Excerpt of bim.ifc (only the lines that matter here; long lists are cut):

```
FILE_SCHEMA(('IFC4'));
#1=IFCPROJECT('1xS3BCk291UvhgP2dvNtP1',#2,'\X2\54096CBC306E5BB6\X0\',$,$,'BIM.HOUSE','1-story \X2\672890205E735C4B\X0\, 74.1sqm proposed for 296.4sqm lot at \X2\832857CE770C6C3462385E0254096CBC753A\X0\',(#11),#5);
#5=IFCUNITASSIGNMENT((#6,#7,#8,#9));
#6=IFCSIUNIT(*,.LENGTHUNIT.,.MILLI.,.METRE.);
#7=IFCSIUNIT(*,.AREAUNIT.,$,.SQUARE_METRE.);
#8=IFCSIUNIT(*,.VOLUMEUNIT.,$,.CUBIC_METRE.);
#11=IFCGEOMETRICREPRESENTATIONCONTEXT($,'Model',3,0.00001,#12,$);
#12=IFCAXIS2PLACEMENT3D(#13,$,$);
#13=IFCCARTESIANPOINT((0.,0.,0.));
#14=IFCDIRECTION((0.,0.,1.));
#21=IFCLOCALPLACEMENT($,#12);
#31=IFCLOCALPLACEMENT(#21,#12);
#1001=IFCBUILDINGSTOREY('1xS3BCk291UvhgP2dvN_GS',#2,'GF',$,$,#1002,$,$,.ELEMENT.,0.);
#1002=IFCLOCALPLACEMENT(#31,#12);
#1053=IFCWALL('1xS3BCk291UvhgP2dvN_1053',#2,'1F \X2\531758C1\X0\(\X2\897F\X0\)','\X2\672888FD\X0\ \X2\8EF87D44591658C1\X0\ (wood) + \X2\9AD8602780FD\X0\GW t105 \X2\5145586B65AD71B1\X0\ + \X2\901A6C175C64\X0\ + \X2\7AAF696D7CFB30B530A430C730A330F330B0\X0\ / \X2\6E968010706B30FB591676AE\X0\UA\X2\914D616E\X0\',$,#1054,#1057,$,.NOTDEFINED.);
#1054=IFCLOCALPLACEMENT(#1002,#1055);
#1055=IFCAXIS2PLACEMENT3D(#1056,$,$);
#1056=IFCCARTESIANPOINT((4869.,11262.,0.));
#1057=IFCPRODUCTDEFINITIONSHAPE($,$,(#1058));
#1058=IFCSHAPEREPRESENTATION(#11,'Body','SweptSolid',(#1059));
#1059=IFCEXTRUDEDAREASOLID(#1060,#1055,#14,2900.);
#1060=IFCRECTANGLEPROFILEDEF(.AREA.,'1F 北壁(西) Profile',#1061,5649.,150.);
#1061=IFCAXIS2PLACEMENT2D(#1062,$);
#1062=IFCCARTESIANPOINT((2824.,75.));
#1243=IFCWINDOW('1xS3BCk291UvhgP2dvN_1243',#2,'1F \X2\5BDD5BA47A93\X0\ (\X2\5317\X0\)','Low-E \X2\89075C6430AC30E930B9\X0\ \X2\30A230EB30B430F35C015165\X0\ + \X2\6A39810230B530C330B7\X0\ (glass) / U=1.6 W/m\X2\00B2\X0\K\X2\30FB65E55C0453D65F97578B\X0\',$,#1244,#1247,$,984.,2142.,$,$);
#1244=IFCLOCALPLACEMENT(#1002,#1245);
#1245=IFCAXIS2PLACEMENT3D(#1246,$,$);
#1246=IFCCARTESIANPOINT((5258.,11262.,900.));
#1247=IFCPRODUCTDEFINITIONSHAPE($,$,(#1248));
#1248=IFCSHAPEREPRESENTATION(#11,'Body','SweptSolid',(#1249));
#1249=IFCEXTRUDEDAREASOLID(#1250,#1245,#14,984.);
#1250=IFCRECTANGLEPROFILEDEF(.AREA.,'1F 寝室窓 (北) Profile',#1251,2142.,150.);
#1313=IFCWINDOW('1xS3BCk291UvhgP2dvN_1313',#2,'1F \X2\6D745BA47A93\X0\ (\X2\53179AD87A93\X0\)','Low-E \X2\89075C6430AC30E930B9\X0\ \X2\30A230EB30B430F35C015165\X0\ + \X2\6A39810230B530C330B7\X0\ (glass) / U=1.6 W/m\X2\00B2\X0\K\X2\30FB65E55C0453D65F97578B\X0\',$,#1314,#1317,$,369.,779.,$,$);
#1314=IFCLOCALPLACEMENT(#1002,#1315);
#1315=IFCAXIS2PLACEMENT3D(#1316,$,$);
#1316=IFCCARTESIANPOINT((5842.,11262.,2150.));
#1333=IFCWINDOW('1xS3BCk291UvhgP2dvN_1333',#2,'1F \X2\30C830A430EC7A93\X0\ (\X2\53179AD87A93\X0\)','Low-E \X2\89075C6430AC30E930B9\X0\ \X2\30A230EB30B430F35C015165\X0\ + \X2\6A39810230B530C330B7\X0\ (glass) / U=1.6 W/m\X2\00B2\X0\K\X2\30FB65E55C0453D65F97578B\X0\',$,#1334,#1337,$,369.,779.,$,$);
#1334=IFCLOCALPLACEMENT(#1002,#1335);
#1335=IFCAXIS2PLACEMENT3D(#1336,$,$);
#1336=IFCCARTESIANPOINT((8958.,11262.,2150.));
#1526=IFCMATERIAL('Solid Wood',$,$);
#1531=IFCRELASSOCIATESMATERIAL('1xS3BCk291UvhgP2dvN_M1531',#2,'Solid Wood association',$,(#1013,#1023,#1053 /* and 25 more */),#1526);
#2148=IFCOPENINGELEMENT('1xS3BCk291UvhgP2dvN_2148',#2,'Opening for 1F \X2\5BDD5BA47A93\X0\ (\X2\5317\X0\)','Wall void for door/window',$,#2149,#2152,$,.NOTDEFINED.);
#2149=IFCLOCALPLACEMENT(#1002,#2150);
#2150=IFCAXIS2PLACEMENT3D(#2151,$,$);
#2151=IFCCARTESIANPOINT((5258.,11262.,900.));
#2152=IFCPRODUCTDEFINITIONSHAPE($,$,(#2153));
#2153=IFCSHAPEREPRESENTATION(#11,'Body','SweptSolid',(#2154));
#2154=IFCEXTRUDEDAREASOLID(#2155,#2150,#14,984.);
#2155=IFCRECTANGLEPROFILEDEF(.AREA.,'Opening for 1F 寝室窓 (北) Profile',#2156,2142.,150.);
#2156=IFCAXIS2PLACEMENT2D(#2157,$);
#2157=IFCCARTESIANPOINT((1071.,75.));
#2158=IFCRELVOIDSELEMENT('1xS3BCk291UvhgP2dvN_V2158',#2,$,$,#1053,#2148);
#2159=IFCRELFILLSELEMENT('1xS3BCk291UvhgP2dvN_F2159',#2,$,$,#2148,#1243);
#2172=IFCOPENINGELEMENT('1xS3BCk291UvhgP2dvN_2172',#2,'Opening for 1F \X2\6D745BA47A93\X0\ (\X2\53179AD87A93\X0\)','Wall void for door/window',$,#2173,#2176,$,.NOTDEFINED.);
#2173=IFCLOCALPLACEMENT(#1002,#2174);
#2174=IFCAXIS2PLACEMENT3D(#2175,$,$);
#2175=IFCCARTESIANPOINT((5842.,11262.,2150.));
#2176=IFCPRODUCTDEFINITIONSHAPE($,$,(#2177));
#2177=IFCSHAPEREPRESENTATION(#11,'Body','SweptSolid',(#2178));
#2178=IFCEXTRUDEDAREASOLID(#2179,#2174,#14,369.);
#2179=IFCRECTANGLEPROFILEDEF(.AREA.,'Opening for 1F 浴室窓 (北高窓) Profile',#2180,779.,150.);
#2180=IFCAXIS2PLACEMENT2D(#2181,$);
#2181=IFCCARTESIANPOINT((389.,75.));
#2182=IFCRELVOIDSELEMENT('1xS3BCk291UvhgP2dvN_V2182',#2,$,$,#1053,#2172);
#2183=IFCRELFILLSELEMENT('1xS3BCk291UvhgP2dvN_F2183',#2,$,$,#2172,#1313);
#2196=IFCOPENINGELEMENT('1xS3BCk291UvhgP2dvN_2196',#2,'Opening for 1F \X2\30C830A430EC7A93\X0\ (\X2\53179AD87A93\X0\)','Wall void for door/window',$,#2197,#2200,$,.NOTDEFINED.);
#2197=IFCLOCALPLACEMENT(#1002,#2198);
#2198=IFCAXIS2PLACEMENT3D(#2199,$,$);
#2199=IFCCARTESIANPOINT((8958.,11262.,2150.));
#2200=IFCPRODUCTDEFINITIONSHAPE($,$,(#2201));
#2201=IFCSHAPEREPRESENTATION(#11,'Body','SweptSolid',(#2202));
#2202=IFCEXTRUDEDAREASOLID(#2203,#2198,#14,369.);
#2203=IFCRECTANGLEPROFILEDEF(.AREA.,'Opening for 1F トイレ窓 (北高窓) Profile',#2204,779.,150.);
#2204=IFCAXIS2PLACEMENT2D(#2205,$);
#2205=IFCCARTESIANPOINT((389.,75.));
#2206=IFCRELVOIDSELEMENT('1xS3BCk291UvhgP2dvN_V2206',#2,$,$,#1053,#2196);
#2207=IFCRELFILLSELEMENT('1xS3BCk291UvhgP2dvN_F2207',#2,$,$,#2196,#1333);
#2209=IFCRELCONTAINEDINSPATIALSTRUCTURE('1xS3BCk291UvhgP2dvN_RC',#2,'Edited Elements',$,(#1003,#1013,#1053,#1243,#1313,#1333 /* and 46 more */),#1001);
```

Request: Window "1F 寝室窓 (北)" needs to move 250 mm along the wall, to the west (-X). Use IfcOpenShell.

```python
import ifcopenshell
import ifcopenshell.api.geometry
import ifcopenshell.util.placement

model = ifcopenshell.open("bim.ifc")

window = model.by_guid("1xS3BCk291UvhgP2dvN_1243")
opening = window.FillsVoids[0].RelatingOpeningElement
wall = opening.VoidsElements[0].RelatingBuildingElement

wall_matrix = ifcopenshell.util.placement.get_local_placement(wall.ObjectPlacement)
shift = wall_matrix[:3, 0] * -250.0
before = ifcopenshell.util.placement.get_local_placement(window.ObjectPlacement)[:3, 3].copy()

# The window is not placed relative to its opening, so move both.
for product in (opening, window):
    matrix = ifcopenshell.util.placement.get_local_placement(product.ObjectPlacement)
    matrix[:3, 3] += shift
    ifcopenshell.api.geometry.edit_object_placement(model, product=product, matrix=matrix, is_si=False)

after = ifcopenshell.util.placement.get_local_placement(window.ObjectPlacement)[:3, 3]
print("window moved by", (after - before).round(3) + 0.0)

model.write("bim_v2.ifc")
```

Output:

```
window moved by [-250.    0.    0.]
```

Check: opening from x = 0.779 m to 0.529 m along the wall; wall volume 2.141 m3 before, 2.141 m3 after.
